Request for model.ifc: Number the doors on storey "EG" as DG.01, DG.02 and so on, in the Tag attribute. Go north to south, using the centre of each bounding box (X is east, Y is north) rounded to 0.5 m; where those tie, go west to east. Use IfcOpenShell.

First a look at what the model holds.

```python
import ifcopenshell
import ifcopenshell.util.element
import ifcopenshell.util.placement

model = ifcopenshell.open("model.ifc")
print(model.schema)
storey = next(s for s in model.by_type("IfcBuildingStorey") if s.Name == "EG")
doors = [e for e in ifcopenshell.util.element.get_decomposition(storey) if e.is_a("IfcDoor")]
for e in sorted(doors, key=lambda e: e.id()):
    origin = ifcopenshell.util.placement.get_local_placement(e.ObjectPlacement)[:3, 3]
    print(e.id(), e.Tag, e.Name, origin.round(2) + 0.0, sep=" | ")
```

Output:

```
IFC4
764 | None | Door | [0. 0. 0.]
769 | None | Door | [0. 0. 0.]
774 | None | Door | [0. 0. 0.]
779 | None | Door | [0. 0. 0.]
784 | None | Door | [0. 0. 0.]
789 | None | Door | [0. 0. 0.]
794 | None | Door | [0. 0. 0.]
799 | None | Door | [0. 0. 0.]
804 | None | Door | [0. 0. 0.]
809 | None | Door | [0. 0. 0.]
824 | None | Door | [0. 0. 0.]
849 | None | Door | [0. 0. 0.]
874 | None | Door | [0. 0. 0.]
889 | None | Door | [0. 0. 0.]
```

```python
import ifcopenshell
import ifcopenshell.geom
import ifcopenshell.util.element
import ifcopenshell.util.shape

model = ifcopenshell.open("model.ifc")
settings = ifcopenshell.geom.settings()
settings.set("use-world-coords", True)


def centre(element):
    shape = ifcopenshell.geom.create_shape(settings, element)
    return ifcopenshell.util.shape.get_bbox_centroid(shape.geometry)


storey = next(s for s in model.by_type("IfcBuildingStorey") if s.Name == "EG")
doors = [e for e in ifcopenshell.util.element.get_decomposition(storey) if e.is_a("IfcDoor")]

# Insertion points can sit at a corner or the storey origin, so sort by the geometry (in metres).
centres = {e: centre(e) for e in doors}
doors.sort(key=lambda e: (-round(centres[e][1] / 0.5), centres[e][0]))

for i, e in enumerate(doors, start=1):
    number = f"DG.{i:02d}"
    e.Tag = number
    print(e.id(), number)

model.write("model_edited.ifc")
```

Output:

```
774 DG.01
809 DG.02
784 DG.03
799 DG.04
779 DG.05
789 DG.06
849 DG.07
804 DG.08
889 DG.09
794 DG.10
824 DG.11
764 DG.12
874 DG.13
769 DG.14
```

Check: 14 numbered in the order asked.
